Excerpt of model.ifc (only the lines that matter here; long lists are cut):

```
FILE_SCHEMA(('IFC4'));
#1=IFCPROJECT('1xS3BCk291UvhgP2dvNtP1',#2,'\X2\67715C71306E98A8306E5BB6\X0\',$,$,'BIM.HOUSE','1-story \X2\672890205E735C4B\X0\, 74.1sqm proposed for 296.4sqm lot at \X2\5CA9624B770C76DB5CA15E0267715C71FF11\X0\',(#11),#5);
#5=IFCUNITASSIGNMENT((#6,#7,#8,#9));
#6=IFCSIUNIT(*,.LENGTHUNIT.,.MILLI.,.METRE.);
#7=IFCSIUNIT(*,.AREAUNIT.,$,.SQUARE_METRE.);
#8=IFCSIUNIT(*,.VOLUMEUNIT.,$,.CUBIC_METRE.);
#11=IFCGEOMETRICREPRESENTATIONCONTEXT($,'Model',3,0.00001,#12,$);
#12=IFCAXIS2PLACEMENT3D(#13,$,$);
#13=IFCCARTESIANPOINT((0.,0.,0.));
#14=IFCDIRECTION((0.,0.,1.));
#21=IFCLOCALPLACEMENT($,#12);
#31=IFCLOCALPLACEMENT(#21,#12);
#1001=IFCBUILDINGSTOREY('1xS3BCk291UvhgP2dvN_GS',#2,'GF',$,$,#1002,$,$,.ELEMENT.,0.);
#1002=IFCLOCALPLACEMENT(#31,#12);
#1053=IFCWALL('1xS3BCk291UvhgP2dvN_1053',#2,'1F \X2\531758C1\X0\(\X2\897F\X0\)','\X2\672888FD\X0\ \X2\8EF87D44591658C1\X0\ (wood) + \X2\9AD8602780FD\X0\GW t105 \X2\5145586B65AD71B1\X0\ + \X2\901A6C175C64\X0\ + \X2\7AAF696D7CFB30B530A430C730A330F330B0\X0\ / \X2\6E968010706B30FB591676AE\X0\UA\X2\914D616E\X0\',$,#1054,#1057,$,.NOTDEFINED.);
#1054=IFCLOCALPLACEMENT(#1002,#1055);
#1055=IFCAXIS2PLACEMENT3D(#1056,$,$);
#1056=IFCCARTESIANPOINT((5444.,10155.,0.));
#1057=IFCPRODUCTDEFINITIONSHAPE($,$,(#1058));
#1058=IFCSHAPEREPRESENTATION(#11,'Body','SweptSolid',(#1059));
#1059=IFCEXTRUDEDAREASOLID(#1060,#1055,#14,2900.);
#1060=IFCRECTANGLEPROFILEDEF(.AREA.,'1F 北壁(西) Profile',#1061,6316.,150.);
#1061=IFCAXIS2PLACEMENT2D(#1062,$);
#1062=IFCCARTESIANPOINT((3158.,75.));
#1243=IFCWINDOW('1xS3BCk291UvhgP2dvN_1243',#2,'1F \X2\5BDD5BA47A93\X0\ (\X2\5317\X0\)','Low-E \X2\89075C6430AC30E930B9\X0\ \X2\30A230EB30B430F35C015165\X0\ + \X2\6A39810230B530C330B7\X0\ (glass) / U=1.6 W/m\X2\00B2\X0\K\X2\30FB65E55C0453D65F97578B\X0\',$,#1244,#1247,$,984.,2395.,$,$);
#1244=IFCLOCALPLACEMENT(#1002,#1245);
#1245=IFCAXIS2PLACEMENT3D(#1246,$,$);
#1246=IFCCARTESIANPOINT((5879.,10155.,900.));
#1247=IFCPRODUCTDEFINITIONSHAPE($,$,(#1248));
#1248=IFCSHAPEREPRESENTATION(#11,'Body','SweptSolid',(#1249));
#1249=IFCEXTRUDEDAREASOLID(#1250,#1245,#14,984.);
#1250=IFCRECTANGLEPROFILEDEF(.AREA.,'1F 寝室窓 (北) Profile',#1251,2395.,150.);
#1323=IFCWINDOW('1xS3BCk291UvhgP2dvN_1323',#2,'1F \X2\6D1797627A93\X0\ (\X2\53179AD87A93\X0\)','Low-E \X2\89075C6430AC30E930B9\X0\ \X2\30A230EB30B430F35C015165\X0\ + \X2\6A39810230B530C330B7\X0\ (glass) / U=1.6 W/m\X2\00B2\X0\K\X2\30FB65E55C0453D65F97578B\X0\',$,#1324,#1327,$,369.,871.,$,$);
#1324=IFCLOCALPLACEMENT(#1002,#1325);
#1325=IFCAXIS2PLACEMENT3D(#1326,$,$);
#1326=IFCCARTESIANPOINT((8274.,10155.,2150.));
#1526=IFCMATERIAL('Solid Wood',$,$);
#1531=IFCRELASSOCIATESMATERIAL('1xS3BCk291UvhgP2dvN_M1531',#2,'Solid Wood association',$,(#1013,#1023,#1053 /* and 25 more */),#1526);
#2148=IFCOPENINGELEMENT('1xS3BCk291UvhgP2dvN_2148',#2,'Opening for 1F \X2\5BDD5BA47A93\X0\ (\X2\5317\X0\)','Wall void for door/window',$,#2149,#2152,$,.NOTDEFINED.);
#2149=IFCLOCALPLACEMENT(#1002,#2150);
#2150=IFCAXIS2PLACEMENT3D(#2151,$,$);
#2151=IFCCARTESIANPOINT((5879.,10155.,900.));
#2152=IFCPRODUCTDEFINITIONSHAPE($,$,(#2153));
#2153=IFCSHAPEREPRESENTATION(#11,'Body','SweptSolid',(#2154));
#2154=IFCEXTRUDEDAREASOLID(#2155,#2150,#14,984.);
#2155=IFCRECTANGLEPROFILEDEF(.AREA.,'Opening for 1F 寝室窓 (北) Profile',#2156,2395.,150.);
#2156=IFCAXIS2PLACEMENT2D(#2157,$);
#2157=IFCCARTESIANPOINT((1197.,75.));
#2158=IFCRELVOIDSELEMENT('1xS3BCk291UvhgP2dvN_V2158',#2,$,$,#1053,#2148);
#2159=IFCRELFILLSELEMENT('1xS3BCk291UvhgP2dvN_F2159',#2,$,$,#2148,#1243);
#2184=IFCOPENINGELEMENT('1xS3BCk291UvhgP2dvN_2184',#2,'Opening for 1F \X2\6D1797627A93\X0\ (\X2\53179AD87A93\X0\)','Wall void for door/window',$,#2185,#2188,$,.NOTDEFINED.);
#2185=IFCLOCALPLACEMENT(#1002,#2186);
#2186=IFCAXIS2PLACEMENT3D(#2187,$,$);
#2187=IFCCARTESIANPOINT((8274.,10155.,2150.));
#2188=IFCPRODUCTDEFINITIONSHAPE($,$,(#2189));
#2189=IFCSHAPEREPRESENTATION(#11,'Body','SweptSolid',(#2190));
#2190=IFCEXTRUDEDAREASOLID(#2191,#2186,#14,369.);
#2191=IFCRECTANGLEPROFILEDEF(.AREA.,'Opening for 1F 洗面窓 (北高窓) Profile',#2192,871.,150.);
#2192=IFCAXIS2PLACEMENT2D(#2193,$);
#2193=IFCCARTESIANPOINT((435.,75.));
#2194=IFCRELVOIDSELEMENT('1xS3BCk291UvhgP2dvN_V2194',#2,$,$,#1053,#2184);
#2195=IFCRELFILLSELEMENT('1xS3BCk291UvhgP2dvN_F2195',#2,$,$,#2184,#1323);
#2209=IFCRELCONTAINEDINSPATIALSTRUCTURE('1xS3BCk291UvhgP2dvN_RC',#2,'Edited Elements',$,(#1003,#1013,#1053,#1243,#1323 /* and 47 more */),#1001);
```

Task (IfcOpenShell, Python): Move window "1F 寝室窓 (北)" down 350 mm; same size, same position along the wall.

```python
import numpy as np
import ifcopenshell
import ifcopenshell.api.geometry
import ifcopenshell.util.placement
import ifcopenshell.util.unit

model = ifcopenshell.open("model.ifc")
unit_scale = ifcopenshell.util.unit.calculate_unit_scale(model)

window = model.by_guid("1xS3BCk291UvhgP2dvN_1243")
opening = window.FillsVoids[0].RelatingOpeningElement
dz = -350.0

shift = np.array([0.0, 0.0, dz])
# The window is not placed relative to its opening, so move both.
for product in (opening, window):
    matrix = ifcopenshell.util.placement.get_local_placement(product.ObjectPlacement)
    matrix[:3, 3] += shift
    ifcopenshell.api.geometry.edit_object_placement(model, product=product, matrix=matrix, is_si=False)

print(f"moved by {dz * unit_scale:+.3f} m")

model.write("model_edited.ifc")
```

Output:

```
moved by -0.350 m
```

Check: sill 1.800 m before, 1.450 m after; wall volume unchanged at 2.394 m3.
